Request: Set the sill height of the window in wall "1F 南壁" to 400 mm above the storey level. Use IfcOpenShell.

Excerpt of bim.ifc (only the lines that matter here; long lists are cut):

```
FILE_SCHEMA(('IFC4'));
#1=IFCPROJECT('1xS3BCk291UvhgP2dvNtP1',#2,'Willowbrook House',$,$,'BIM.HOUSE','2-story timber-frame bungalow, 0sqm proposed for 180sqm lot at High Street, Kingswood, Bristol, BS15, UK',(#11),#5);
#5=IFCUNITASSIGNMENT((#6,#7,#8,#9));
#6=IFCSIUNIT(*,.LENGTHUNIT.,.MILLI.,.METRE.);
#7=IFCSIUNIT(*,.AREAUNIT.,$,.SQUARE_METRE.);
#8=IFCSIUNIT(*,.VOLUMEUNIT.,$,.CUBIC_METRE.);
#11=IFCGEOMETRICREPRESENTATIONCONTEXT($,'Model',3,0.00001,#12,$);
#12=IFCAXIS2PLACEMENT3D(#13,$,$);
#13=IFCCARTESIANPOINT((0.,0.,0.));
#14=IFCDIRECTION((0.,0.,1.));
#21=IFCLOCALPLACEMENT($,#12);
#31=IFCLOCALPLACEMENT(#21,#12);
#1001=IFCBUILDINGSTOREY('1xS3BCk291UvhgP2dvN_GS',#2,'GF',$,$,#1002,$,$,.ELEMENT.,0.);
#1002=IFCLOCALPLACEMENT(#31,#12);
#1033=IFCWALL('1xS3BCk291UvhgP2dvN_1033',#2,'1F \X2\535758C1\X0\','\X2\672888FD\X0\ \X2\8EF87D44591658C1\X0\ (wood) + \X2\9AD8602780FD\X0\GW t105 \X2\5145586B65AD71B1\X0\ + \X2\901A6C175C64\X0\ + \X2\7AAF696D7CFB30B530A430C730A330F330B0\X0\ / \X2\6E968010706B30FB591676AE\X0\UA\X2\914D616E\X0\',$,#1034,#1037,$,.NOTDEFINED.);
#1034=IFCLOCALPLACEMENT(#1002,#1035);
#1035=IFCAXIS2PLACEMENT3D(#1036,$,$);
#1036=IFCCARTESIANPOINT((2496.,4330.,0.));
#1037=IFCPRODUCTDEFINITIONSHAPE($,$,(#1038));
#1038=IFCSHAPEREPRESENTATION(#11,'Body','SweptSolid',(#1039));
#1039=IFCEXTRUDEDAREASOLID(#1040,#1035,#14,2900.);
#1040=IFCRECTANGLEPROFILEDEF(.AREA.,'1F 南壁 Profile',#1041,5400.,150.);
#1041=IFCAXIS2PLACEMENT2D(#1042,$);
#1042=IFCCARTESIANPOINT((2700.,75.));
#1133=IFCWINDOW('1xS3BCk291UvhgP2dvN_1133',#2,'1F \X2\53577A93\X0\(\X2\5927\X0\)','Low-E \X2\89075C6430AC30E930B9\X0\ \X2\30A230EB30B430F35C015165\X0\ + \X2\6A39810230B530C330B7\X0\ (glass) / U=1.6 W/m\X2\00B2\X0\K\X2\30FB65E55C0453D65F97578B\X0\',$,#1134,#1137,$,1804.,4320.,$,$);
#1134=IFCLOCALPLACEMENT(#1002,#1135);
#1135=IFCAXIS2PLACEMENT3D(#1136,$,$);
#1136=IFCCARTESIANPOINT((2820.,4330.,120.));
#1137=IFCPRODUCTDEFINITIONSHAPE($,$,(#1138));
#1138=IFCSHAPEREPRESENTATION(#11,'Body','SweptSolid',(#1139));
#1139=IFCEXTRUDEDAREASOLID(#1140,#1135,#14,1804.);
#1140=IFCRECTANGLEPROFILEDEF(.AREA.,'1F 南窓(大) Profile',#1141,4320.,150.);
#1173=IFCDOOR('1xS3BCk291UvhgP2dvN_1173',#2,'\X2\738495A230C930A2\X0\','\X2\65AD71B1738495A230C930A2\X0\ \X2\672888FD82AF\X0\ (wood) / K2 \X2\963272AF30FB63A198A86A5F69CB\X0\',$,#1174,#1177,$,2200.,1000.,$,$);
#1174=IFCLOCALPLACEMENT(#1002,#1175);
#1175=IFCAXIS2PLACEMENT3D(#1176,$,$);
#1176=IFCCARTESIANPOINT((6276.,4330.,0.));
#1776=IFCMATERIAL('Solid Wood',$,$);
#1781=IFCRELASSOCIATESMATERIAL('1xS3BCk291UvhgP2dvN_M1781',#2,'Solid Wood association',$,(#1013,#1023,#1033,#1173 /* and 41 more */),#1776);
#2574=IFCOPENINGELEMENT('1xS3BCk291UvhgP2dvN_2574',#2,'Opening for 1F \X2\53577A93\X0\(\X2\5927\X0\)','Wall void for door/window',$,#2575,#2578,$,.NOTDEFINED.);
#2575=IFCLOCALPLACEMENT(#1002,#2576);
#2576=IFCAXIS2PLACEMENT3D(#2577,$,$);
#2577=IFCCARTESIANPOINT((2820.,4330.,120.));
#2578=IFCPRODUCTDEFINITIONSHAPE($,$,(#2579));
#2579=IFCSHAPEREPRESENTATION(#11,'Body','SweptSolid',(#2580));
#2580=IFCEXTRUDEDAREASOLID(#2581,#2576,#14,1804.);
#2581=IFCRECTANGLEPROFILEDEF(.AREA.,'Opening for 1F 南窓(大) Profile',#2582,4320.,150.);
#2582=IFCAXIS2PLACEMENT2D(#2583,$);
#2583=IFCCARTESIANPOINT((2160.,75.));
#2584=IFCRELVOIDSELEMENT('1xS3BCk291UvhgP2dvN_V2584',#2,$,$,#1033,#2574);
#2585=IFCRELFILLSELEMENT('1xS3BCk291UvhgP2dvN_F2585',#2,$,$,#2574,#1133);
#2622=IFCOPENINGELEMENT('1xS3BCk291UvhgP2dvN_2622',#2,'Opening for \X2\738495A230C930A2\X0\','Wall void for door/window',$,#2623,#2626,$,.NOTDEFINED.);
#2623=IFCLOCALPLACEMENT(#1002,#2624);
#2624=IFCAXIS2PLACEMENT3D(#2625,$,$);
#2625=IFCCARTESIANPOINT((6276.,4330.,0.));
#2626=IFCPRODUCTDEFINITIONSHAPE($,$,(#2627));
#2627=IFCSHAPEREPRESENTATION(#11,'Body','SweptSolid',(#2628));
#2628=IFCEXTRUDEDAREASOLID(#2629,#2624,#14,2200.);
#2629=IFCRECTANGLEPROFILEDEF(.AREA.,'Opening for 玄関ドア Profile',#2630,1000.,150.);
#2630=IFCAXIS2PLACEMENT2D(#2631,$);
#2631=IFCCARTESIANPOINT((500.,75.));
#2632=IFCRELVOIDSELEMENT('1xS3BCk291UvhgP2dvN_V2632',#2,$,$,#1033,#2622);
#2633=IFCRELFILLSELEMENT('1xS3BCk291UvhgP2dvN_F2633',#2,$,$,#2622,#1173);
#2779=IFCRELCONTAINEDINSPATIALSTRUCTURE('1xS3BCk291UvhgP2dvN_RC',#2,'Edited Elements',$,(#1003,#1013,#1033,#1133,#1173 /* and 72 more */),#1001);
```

```python
import numpy as np
import ifcopenshell
import ifcopenshell.api.geometry
import ifcopenshell.geom
import ifcopenshell.util.element
import ifcopenshell.util.placement
import ifcopenshell.util.shape
import ifcopenshell.util.unit

model = ifcopenshell.open("bim.ifc")
unit_scale = ifcopenshell.util.unit.calculate_unit_scale(model)

window = model.by_id(1133)
opening = window.FillsVoids[0].RelatingOpeningElement
storey = ifcopenshell.util.element.get_container(window, ifc_class="IfcBuildingStorey")
level = ifcopenshell.util.placement.get_local_placement(storey.ObjectPlacement)[2, 3]

# The opening's origin need not be at the sill, so measure its lowest point.
shape = ifcopenshell.geom.create_shape(ifcopenshell.geom.settings(), opening)
bottom = ifcopenshell.util.shape.get_shape_bottom_elevation(shape, shape.geometry) / unit_scale
dz = level + 400.0 - bottom

shift = np.array([0.0, 0.0, dz])
# The window is not placed relative to its opening, so move both.
for product in (opening, window):
    matrix = ifcopenshell.util.placement.get_local_placement(product.ObjectPlacement)
    matrix[:3, 3] += shift
    ifcopenshell.api.geometry.edit_object_placement(model, product=product, matrix=matrix, is_si=False)

print(f"moved by {dz * unit_scale:+.3f} m")

model.write("bim-out.ifc")
```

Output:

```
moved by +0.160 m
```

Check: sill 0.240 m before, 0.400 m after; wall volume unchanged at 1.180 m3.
